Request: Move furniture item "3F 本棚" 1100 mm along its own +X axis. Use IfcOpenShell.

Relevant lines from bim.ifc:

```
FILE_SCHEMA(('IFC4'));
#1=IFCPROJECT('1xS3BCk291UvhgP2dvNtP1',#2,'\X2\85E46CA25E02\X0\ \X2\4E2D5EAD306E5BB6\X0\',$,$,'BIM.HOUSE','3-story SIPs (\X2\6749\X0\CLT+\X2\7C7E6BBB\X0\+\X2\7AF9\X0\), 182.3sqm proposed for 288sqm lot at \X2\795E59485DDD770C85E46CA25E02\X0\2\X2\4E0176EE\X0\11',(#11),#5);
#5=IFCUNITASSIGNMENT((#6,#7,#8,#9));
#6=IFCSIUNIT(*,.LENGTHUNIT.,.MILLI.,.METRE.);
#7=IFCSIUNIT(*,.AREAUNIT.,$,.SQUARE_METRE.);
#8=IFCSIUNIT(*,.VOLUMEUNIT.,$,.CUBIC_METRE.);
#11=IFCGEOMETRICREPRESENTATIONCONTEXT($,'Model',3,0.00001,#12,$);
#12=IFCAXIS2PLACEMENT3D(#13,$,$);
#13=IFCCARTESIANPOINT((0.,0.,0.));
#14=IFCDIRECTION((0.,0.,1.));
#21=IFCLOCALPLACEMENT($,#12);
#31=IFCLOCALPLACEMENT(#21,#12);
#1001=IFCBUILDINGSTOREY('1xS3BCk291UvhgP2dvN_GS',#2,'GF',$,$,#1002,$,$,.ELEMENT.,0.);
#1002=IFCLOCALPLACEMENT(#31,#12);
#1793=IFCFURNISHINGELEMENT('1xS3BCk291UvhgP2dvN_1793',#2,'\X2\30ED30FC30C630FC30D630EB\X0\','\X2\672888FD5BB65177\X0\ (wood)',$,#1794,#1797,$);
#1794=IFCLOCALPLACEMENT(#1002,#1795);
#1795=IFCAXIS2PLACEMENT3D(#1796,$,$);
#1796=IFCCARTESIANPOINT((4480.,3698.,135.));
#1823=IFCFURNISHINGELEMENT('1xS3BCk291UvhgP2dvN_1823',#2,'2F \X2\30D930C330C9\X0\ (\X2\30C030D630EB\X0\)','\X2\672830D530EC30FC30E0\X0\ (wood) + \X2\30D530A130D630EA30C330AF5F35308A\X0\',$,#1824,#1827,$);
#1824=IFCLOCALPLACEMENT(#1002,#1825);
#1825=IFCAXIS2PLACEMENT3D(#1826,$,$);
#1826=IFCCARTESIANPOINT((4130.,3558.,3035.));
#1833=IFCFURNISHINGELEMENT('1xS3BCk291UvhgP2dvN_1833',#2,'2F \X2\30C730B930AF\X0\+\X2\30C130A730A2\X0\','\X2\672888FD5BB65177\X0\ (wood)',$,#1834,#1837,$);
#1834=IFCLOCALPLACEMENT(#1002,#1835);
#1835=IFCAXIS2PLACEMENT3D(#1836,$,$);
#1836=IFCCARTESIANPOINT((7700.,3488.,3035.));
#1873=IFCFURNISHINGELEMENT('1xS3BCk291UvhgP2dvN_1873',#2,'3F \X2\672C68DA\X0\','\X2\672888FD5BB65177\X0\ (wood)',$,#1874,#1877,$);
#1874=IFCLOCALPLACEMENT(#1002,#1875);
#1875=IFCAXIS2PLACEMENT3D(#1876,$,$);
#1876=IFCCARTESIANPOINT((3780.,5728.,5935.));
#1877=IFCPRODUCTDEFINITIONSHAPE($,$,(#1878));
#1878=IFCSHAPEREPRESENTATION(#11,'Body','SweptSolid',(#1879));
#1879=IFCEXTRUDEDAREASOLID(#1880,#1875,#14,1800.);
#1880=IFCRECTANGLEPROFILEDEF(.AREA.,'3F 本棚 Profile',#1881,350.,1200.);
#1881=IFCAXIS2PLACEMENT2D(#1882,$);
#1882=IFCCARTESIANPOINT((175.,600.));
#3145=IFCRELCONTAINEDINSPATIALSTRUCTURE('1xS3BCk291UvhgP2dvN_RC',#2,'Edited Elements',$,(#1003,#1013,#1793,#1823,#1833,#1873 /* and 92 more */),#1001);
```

```python
import ifcopenshell
import ifcopenshell.api.geometry
import ifcopenshell.util.placement
import ifcopenshell.util.unit

model = ifcopenshell.open("bim.ifc")
unit_scale = ifcopenshell.util.unit.calculate_unit_scale(model)

item = model.by_guid("1xS3BCk291UvhgP2dvN_1873")
matrix = ifcopenshell.util.placement.get_local_placement(item.ObjectPlacement)
matrix[:3, 3] += matrix[:3, 0] * 1.1 / unit_scale
ifcopenshell.api.geometry.edit_object_placement(model, product=item, matrix=matrix, is_si=False)

print(ifcopenshell.util.placement.get_local_placement(item.ObjectPlacement).round(3) + 0.0)

model.write("bim-out.ifc")
```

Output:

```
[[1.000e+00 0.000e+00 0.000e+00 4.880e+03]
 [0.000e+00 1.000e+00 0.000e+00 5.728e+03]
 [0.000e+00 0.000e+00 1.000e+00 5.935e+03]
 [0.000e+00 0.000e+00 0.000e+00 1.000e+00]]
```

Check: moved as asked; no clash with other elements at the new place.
